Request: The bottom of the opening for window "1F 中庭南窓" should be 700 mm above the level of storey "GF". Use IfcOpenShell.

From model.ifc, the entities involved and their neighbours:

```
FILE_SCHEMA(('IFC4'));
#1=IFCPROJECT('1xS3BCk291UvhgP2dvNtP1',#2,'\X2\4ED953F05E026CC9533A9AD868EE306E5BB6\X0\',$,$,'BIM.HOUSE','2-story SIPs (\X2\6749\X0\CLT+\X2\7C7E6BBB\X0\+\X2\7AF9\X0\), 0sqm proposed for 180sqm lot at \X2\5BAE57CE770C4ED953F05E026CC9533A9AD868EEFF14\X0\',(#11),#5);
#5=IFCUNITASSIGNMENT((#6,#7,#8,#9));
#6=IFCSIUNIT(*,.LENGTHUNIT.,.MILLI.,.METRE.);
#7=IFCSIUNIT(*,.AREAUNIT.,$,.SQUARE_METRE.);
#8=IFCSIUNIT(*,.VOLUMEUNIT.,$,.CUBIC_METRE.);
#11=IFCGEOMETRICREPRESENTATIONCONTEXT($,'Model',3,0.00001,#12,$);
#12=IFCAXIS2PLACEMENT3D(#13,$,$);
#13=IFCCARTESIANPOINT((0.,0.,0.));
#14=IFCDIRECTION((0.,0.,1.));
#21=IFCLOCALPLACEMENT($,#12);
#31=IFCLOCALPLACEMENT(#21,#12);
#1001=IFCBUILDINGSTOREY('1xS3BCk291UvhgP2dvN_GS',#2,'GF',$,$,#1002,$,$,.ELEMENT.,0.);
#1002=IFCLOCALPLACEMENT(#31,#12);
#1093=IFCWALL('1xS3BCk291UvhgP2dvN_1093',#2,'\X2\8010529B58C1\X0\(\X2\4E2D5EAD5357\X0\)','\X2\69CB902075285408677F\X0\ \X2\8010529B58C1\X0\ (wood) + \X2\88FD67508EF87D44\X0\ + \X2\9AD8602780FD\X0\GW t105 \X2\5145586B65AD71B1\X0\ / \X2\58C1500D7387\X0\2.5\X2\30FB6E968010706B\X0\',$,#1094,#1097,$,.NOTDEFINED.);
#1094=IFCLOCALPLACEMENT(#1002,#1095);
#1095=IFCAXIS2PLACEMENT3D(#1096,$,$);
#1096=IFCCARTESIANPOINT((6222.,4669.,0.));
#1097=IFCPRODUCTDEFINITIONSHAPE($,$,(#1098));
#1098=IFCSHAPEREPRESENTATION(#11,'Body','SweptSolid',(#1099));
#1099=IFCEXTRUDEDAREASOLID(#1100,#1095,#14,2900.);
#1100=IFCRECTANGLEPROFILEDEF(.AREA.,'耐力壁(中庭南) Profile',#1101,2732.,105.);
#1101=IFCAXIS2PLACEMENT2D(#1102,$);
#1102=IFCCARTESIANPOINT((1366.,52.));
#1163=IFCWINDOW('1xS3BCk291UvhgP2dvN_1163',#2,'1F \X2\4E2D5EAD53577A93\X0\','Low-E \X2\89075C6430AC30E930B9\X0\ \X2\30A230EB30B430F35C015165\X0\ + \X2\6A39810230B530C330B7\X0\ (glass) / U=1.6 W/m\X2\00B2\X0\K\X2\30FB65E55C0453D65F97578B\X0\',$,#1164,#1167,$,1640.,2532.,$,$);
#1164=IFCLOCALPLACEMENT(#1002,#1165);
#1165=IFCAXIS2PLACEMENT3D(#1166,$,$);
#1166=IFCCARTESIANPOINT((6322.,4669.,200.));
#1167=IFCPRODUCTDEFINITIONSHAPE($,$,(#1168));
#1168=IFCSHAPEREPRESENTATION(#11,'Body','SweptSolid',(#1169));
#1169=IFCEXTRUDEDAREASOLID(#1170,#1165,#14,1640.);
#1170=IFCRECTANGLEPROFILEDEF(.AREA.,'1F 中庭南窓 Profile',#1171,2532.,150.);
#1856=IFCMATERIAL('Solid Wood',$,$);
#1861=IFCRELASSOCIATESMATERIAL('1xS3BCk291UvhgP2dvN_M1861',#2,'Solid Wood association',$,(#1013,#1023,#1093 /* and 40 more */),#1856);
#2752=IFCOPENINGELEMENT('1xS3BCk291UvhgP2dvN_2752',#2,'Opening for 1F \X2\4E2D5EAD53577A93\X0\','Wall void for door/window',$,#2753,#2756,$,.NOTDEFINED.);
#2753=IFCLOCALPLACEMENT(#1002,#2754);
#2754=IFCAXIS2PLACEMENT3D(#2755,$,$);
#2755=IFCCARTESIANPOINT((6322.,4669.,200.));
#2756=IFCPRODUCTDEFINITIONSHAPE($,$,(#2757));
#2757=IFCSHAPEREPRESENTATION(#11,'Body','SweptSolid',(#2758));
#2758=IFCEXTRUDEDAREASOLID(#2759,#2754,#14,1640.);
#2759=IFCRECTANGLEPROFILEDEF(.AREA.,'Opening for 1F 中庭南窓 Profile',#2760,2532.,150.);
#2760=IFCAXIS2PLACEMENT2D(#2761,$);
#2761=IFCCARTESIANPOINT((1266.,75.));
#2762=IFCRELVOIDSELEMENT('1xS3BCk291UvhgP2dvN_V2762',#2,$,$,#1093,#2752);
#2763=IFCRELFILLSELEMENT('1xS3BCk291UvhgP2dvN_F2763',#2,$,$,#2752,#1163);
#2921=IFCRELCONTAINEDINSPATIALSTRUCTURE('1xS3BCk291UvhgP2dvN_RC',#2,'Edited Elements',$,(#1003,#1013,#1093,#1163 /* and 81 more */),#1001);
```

```python
import numpy as np
import ifcopenshell
import ifcopenshell.api.geometry
import ifcopenshell.geom
import ifcopenshell.util.element
import ifcopenshell.util.placement
import ifcopenshell.util.shape
import ifcopenshell.util.unit

model = ifcopenshell.open("model.ifc")
unit_scale = ifcopenshell.util.unit.calculate_unit_scale(model)

window = model.by_id(1163)
opening = window.FillsVoids[0].RelatingOpeningElement
storey = ifcopenshell.util.element.get_container(window, ifc_class="IfcBuildingStorey")
level = ifcopenshell.util.placement.get_local_placement(storey.ObjectPlacement)[2, 3]

# The opening's origin need not be at the sill, so measure its lowest point.
shape = ifcopenshell.geom.create_shape(ifcopenshell.geom.settings(), opening)
bottom = ifcopenshell.util.shape.get_shape_bottom_elevation(shape, shape.geometry) / unit_scale
dz = level + 700.0 - bottom

shift = np.array([0.0, 0.0, dz])
# The window is not placed relative to its opening, so move both.
for product in (opening, window):
    matrix = ifcopenshell.util.placement.get_local_placement(product.ObjectPlacement)
    matrix[:3, 3] += shift
    ifcopenshell.api.geometry.edit_object_placement(model, product=product, matrix=matrix, is_si=False)

print(f"moved by {dz * unit_scale:+.3f} m")

model.write("model_v2.ifc")
```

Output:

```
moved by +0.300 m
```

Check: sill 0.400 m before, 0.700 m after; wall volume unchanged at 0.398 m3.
